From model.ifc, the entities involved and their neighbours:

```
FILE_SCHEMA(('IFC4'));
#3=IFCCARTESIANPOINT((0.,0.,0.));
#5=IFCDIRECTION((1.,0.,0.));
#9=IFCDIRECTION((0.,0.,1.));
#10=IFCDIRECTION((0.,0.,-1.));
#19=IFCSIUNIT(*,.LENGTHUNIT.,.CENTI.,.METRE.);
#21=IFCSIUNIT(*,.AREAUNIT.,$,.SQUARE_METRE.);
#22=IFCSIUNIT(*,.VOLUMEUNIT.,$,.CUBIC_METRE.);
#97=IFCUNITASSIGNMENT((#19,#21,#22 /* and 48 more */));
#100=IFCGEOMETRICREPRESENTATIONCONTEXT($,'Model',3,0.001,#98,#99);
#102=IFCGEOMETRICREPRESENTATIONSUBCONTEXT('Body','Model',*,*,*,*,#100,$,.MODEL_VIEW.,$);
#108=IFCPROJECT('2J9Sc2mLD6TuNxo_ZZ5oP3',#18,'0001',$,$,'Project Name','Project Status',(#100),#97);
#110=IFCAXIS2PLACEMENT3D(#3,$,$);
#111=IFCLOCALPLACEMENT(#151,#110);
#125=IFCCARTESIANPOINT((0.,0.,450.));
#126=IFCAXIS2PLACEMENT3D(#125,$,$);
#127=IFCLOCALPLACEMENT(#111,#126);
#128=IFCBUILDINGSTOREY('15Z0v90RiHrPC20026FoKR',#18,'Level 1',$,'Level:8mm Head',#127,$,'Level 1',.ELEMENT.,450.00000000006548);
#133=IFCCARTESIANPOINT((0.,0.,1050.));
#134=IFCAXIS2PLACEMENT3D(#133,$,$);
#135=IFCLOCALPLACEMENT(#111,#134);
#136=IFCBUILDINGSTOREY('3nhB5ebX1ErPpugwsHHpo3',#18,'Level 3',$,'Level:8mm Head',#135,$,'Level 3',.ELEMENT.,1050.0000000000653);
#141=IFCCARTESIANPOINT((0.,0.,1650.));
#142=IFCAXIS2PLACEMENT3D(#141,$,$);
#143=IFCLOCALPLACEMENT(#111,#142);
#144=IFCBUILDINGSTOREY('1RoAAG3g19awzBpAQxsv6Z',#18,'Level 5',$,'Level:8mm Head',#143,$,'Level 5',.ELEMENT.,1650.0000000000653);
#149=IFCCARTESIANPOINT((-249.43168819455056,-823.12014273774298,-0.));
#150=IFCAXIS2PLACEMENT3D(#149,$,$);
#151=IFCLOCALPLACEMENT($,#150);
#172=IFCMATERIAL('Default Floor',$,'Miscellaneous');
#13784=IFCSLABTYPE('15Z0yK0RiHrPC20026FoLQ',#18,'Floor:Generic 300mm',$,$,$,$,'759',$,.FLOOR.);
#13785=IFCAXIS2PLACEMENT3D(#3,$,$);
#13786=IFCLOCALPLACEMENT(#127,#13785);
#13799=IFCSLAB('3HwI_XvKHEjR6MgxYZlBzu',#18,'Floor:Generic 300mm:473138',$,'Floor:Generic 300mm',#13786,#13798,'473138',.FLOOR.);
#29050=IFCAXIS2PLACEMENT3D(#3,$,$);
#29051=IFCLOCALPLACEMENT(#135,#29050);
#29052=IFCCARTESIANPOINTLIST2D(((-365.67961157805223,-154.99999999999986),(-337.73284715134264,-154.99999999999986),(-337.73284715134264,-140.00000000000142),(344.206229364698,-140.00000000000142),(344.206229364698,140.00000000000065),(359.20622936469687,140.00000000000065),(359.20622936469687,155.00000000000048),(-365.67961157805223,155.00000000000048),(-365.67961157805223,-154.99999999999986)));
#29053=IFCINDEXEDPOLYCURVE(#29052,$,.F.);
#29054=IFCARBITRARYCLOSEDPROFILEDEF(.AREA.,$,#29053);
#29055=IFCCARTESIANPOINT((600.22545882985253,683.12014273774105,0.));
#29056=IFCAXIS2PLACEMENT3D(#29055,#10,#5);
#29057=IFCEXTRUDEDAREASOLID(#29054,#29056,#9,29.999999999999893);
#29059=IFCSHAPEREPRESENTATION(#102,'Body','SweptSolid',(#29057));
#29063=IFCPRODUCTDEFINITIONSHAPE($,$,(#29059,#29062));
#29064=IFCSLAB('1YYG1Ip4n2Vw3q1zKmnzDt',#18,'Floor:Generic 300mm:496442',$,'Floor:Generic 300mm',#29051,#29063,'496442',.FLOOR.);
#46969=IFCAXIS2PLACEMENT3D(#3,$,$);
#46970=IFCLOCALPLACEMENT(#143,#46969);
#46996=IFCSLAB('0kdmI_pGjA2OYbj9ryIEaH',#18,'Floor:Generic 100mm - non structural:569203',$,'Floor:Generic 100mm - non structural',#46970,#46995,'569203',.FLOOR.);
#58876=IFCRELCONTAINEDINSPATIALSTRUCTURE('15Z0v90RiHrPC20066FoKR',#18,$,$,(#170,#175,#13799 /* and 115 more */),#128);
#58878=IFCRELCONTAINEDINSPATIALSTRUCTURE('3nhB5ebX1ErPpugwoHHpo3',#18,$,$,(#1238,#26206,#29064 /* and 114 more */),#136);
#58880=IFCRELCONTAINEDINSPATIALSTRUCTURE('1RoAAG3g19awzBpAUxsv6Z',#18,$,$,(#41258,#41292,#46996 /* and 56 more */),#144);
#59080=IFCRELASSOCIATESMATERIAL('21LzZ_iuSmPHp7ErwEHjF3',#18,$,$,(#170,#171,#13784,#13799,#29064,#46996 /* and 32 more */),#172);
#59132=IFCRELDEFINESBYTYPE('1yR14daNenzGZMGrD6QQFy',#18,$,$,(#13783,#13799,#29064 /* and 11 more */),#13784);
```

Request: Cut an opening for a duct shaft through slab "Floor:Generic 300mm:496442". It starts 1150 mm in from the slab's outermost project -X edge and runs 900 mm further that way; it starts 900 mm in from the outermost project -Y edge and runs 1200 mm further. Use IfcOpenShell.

```python
import numpy as np
import ifcopenshell
import ifcopenshell.api.feature
import ifcopenshell.api.geometry
import ifcopenshell.api.root
import ifcopenshell.geom
import ifcopenshell.util.placement
import ifcopenshell.util.representation
import ifcopenshell.util.shape
import ifcopenshell.util.unit

model = ifcopenshell.open("model.ifc")
unit_scale = ifcopenshell.util.unit.calculate_unit_scale(model)
settings = ifcopenshell.geom.settings()


def volume(element):
    """Net volume in cubic metres, openings subtracted."""
    shape = ifcopenshell.geom.create_shape(settings, element)
    return ifcopenshell.util.shape.get_volume(shape.geometry)


slab = model.by_guid("1YYG1Ip4n2Vw3q1zKmnzDt")
before = volume(slab)

# Extent in the slab's own axes, in metres. The edges named are its -X and -Y sides.
slab_shape = ifcopenshell.geom.create_shape(settings, slab)
vertices = ifcopenshell.util.shape.get_vertices(slab_shape.geometry)
x_min, y_min, bottom = vertices.min(axis=0)
top = vertices[:, 2].max()

opening = ifcopenshell.api.root.create_entity(model, ifc_class="IfcOpeningElement", name="Duct shaft opening", predefined_type="OPENING")
context = ifcopenshell.util.representation.get_context(model, "Model", "Body", "MODEL_VIEW")
width, depth = 0.9, 1.2
outline = [(0.0, 0.0), (width, 0.0), (width, depth), (0.0, depth), (0.0, 0.0)]
# Overshoot both faces by 50 mm so the cut is clean.
shape = ifcopenshell.api.geometry.add_slab_representation(
    model, context=context, depth=top - bottom + 0.1, polyline=outline
)
ifcopenshell.api.geometry.assign_representation(model, product=opening, representation=shape)

matrix = ifcopenshell.util.placement.get_local_placement(slab.ObjectPlacement)
matrix[:, 3] = matrix @ np.append(np.array([x_min + 1.15, y_min + 0.9, bottom - 0.05]) / unit_scale, 1.0)
ifcopenshell.api.geometry.edit_object_placement(model, product=opening, matrix=matrix, is_si=False)
ifcopenshell.api.feature.add_feature(model, feature=opening, element=slab)

after = volume(slab)

print(f"slab volume {before:.3f} -> {after:.3f} m3")

model.write("model_updated.ifc")
```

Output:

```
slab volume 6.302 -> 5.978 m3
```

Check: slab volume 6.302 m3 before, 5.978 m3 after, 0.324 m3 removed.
